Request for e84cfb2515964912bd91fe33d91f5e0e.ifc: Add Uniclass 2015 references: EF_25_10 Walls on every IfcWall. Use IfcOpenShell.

First a look at what the model holds.

```python
import ifcopenshell

model = ifcopenshell.open("e84cfb2515964912bd91fe33d91f5e0e.ifc")
print(model.schema)
print("classifications:", [c.Name for c in model.by_type("IfcClassification")])
for ifc_class in ("IfcDoor", "IfcRoof", "IfcStair", "IfcWall", "IfcWindow"):
    print(ifc_class, len(model.by_type(ifc_class)))
```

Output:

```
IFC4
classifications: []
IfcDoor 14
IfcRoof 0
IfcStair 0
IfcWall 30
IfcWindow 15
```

```python
import ifcopenshell
import ifcopenshell.api.classification

model = ifcopenshell.open("e84cfb2515964912bd91fe33d91f5e0e.ifc")

system = ifcopenshell.api.classification.add_classification(model, classification="Uniclass 2015")

codes = {
    "IfcWall": ("EF_25_10", "Walls"),
}
for ifc_class, (code, name) in codes.items():
    products = model.by_type(ifc_class)
    ifcopenshell.api.classification.add_reference(
        model, products=products, classification=system, identification=code, name=name
    )
    print(code, len(products))

model.write("e84cfb2515964912bd91fe33d91f5e0e_rev.ifc")
```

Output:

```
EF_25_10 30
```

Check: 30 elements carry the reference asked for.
